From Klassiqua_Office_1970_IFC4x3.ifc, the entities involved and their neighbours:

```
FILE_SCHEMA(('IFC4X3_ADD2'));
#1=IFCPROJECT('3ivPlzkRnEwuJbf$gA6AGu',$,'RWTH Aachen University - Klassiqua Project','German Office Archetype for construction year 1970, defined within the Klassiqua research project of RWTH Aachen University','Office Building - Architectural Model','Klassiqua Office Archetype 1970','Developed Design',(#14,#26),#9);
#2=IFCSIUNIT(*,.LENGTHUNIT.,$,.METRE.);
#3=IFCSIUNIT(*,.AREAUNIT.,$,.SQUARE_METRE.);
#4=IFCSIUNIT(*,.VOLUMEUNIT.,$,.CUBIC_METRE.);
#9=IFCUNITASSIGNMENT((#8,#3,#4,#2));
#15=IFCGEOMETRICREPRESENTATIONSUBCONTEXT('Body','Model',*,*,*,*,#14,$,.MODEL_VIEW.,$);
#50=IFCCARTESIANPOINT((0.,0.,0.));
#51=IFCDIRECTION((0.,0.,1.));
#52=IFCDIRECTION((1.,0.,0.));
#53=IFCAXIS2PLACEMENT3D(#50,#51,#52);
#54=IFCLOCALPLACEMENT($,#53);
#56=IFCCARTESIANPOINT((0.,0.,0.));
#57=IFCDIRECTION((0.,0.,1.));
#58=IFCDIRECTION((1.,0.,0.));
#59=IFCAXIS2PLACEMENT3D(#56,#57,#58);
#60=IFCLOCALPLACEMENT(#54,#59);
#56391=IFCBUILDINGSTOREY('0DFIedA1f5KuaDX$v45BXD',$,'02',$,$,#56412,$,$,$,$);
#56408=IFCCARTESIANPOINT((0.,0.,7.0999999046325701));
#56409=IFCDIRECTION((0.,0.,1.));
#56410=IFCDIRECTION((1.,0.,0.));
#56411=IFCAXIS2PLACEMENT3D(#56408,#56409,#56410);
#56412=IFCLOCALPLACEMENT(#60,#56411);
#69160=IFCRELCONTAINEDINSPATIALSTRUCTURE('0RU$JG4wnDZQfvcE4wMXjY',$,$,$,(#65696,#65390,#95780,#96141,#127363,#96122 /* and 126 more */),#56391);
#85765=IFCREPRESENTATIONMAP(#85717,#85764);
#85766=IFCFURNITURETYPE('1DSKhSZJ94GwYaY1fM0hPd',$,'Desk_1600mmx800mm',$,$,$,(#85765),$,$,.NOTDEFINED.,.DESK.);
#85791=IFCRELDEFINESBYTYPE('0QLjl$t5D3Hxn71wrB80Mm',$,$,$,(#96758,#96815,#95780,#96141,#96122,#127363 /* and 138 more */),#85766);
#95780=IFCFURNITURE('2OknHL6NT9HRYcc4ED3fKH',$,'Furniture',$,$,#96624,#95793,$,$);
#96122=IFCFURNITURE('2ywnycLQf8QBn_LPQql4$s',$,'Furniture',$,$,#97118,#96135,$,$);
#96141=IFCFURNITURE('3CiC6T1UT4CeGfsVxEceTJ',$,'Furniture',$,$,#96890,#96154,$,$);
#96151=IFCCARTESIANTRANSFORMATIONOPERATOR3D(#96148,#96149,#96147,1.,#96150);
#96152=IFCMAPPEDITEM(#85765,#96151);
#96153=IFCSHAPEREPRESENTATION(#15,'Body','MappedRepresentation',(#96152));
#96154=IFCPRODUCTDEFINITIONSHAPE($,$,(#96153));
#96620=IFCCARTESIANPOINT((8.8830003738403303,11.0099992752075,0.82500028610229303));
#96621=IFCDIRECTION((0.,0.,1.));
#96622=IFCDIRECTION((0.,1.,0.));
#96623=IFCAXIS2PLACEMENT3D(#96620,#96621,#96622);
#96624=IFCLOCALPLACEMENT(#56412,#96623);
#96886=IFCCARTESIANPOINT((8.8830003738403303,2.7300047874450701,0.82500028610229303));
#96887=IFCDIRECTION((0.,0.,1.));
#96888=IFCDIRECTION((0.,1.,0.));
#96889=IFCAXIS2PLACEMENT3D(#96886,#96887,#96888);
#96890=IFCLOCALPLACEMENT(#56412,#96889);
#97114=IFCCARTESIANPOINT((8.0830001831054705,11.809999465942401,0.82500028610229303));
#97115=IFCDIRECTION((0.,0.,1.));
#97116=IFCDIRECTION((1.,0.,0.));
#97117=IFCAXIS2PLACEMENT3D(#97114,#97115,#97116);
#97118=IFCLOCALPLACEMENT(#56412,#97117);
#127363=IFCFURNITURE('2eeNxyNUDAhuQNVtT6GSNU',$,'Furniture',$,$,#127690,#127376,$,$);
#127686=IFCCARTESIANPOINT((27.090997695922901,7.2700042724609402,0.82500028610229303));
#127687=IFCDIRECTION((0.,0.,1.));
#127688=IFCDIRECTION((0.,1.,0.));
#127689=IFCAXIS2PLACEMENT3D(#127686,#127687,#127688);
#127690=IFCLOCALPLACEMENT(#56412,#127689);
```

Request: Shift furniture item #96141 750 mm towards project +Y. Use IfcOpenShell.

```python
import ifcopenshell
import ifcopenshell.api.geometry
import ifcopenshell.util.placement
import ifcopenshell.util.unit

model = ifcopenshell.open("Klassiqua_Office_1970_IFC4x3.ifc")
unit_scale = ifcopenshell.util.unit.calculate_unit_scale(model)

item = model.by_guid("3CiC6T1UT4CeGfsVxEceTJ")
matrix = ifcopenshell.util.placement.get_local_placement(item.ObjectPlacement)
matrix[1, 3] += 0.75 / unit_scale
ifcopenshell.api.geometry.edit_object_placement(model, product=item, matrix=matrix, is_si=False)

print(ifcopenshell.util.placement.get_local_placement(item.ObjectPlacement).round(3) + 0.0)

model.write("Klassiqua_Office_1970_IFC4x3-out.ifc")
```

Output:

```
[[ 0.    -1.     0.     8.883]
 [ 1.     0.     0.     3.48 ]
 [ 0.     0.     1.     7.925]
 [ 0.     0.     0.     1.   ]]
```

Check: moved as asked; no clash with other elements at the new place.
